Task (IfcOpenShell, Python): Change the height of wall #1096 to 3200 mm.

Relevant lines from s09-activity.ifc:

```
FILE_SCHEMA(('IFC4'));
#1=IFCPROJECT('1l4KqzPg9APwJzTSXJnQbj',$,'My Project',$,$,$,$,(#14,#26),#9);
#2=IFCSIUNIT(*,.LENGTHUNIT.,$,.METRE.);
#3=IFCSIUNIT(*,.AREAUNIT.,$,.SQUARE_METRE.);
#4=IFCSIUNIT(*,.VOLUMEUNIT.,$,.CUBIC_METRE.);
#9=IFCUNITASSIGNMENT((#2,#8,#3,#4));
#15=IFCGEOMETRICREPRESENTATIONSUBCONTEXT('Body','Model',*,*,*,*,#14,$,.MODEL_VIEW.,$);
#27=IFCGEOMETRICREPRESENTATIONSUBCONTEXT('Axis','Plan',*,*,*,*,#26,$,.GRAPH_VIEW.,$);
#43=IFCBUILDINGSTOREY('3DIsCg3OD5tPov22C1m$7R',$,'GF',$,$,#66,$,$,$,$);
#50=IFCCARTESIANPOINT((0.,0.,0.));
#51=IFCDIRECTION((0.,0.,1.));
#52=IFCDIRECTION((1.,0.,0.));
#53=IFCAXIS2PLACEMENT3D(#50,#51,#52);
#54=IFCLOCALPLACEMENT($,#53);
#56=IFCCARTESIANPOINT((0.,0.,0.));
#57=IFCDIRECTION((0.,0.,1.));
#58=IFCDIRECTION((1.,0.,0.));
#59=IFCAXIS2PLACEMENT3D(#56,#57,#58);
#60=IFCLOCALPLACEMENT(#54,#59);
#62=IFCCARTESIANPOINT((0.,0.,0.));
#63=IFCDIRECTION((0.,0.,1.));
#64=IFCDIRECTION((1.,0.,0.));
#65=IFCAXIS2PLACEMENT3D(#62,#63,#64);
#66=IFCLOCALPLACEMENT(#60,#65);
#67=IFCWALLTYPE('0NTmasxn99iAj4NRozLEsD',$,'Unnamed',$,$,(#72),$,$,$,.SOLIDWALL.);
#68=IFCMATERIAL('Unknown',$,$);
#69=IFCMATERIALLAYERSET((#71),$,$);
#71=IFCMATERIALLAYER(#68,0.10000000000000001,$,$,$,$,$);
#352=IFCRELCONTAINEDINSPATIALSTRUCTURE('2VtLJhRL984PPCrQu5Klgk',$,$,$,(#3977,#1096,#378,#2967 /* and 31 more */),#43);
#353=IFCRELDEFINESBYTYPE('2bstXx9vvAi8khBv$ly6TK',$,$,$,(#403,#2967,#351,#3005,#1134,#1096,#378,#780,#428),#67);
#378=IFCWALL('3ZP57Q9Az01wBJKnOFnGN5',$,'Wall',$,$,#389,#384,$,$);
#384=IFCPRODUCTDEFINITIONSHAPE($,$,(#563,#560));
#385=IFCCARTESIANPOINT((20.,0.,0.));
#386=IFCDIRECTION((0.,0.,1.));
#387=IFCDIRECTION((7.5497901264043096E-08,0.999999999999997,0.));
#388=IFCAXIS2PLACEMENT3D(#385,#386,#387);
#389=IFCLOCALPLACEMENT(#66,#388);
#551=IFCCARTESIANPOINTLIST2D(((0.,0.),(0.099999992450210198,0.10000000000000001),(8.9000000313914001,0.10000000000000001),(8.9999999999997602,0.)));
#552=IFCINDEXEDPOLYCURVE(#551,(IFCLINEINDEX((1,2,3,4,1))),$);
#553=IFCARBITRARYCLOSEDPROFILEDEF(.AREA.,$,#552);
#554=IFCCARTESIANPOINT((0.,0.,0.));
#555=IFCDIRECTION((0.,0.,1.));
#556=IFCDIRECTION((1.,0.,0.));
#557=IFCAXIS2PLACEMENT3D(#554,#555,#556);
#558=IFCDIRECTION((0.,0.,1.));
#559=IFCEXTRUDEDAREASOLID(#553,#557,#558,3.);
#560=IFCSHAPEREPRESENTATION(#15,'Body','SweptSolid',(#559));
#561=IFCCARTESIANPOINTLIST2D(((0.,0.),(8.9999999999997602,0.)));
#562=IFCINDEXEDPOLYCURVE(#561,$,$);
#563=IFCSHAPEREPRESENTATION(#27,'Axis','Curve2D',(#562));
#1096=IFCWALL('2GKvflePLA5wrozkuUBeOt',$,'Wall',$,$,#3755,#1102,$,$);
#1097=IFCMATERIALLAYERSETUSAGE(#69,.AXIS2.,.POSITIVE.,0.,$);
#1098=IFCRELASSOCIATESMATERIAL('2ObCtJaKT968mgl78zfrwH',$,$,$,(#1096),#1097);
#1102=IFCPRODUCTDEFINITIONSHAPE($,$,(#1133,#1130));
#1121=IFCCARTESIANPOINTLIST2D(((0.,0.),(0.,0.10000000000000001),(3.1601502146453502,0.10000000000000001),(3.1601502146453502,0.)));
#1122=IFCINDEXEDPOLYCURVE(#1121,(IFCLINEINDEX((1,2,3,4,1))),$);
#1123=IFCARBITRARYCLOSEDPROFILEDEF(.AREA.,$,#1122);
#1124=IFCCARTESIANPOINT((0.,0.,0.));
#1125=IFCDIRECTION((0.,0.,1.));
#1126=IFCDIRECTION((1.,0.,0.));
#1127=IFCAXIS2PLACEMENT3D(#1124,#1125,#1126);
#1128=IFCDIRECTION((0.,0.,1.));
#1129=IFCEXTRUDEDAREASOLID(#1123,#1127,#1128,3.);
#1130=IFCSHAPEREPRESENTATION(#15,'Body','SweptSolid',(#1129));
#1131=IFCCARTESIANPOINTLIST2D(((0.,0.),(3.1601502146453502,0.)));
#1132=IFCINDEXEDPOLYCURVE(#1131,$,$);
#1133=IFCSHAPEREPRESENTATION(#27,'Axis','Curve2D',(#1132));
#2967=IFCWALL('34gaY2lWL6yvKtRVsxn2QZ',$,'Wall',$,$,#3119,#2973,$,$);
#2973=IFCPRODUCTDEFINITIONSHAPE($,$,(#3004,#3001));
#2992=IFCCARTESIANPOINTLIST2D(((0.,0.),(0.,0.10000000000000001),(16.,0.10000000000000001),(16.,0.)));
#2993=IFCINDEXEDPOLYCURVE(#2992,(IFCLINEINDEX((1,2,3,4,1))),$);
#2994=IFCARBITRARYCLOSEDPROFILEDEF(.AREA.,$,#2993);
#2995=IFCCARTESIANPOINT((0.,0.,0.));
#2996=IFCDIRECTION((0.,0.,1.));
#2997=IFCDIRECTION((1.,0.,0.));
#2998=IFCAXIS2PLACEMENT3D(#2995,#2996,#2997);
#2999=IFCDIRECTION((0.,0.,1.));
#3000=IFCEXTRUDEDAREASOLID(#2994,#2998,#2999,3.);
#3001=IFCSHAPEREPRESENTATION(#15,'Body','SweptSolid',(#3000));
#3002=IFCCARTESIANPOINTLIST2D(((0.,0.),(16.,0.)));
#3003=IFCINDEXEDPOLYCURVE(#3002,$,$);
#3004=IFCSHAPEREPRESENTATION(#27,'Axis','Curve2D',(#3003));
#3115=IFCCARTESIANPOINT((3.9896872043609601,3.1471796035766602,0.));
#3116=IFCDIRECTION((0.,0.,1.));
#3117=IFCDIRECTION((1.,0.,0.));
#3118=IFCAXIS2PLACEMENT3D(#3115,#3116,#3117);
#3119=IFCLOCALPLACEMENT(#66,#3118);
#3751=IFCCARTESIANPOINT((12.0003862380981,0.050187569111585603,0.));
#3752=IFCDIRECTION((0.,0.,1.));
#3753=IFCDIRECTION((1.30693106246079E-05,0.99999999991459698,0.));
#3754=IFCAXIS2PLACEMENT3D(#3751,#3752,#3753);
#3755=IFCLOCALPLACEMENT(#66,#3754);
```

```python
import ifcopenshell
import ifcopenshell.geom
import ifcopenshell.util.representation
import ifcopenshell.util.shape

model = ifcopenshell.open("s09-activity.ifc")
settings = ifcopenshell.geom.settings()


def volume(element):
    """Net volume in cubic metres, openings subtracted."""
    shape = ifcopenshell.geom.create_shape(settings, element)
    return ifcopenshell.util.shape.get_volume(shape.geometry)


wall = model.by_id(1096)
before = volume(wall)

body = ifcopenshell.util.representation.get_representation(wall, "Model", "Body")
solid = body.Items[0]
old_height = solid.Depth
solid.Depth = 3.2
after = volume(wall)

print(f"height {old_height:g} -> {solid.Depth:g}, volume {before:.3f} -> {after:.3f} m3")

model.write("s09-activity_v2.ifc")
```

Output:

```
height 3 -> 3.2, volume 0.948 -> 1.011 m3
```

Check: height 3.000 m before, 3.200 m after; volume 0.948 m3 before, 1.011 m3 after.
